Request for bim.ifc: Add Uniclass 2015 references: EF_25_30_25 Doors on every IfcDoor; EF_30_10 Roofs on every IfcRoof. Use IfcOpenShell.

First a look at what the model holds.

```python
import ifcopenshell

model = ifcopenshell.open("bim.ifc")
print(model.schema)
print("classifications:", [c.Name for c in model.by_type("IfcClassification")])
for ifc_class in ("IfcDoor", "IfcRoof", "IfcStair", "IfcWall", "IfcWindow"):
    print(ifc_class, len(model.by_type(ifc_class)))
```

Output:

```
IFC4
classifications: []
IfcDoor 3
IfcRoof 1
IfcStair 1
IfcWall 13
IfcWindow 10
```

```python
import ifcopenshell
import ifcopenshell.api.classification

model = ifcopenshell.open("bim.ifc")

system = ifcopenshell.api.classification.add_classification(model, classification="Uniclass 2015")

codes = {
    "IfcDoor": ("EF_25_30_25", "Doors"),
    "IfcRoof": ("EF_30_10", "Roofs"),
}
for ifc_class, (code, name) in codes.items():
    products = model.by_type(ifc_class)
    ifcopenshell.api.classification.add_reference(
        model, products=products, classification=system, identification=code, name=name
    )
    print(code, len(products))

model.write("bim_edited.ifc")
```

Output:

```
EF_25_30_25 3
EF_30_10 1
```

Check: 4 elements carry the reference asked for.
